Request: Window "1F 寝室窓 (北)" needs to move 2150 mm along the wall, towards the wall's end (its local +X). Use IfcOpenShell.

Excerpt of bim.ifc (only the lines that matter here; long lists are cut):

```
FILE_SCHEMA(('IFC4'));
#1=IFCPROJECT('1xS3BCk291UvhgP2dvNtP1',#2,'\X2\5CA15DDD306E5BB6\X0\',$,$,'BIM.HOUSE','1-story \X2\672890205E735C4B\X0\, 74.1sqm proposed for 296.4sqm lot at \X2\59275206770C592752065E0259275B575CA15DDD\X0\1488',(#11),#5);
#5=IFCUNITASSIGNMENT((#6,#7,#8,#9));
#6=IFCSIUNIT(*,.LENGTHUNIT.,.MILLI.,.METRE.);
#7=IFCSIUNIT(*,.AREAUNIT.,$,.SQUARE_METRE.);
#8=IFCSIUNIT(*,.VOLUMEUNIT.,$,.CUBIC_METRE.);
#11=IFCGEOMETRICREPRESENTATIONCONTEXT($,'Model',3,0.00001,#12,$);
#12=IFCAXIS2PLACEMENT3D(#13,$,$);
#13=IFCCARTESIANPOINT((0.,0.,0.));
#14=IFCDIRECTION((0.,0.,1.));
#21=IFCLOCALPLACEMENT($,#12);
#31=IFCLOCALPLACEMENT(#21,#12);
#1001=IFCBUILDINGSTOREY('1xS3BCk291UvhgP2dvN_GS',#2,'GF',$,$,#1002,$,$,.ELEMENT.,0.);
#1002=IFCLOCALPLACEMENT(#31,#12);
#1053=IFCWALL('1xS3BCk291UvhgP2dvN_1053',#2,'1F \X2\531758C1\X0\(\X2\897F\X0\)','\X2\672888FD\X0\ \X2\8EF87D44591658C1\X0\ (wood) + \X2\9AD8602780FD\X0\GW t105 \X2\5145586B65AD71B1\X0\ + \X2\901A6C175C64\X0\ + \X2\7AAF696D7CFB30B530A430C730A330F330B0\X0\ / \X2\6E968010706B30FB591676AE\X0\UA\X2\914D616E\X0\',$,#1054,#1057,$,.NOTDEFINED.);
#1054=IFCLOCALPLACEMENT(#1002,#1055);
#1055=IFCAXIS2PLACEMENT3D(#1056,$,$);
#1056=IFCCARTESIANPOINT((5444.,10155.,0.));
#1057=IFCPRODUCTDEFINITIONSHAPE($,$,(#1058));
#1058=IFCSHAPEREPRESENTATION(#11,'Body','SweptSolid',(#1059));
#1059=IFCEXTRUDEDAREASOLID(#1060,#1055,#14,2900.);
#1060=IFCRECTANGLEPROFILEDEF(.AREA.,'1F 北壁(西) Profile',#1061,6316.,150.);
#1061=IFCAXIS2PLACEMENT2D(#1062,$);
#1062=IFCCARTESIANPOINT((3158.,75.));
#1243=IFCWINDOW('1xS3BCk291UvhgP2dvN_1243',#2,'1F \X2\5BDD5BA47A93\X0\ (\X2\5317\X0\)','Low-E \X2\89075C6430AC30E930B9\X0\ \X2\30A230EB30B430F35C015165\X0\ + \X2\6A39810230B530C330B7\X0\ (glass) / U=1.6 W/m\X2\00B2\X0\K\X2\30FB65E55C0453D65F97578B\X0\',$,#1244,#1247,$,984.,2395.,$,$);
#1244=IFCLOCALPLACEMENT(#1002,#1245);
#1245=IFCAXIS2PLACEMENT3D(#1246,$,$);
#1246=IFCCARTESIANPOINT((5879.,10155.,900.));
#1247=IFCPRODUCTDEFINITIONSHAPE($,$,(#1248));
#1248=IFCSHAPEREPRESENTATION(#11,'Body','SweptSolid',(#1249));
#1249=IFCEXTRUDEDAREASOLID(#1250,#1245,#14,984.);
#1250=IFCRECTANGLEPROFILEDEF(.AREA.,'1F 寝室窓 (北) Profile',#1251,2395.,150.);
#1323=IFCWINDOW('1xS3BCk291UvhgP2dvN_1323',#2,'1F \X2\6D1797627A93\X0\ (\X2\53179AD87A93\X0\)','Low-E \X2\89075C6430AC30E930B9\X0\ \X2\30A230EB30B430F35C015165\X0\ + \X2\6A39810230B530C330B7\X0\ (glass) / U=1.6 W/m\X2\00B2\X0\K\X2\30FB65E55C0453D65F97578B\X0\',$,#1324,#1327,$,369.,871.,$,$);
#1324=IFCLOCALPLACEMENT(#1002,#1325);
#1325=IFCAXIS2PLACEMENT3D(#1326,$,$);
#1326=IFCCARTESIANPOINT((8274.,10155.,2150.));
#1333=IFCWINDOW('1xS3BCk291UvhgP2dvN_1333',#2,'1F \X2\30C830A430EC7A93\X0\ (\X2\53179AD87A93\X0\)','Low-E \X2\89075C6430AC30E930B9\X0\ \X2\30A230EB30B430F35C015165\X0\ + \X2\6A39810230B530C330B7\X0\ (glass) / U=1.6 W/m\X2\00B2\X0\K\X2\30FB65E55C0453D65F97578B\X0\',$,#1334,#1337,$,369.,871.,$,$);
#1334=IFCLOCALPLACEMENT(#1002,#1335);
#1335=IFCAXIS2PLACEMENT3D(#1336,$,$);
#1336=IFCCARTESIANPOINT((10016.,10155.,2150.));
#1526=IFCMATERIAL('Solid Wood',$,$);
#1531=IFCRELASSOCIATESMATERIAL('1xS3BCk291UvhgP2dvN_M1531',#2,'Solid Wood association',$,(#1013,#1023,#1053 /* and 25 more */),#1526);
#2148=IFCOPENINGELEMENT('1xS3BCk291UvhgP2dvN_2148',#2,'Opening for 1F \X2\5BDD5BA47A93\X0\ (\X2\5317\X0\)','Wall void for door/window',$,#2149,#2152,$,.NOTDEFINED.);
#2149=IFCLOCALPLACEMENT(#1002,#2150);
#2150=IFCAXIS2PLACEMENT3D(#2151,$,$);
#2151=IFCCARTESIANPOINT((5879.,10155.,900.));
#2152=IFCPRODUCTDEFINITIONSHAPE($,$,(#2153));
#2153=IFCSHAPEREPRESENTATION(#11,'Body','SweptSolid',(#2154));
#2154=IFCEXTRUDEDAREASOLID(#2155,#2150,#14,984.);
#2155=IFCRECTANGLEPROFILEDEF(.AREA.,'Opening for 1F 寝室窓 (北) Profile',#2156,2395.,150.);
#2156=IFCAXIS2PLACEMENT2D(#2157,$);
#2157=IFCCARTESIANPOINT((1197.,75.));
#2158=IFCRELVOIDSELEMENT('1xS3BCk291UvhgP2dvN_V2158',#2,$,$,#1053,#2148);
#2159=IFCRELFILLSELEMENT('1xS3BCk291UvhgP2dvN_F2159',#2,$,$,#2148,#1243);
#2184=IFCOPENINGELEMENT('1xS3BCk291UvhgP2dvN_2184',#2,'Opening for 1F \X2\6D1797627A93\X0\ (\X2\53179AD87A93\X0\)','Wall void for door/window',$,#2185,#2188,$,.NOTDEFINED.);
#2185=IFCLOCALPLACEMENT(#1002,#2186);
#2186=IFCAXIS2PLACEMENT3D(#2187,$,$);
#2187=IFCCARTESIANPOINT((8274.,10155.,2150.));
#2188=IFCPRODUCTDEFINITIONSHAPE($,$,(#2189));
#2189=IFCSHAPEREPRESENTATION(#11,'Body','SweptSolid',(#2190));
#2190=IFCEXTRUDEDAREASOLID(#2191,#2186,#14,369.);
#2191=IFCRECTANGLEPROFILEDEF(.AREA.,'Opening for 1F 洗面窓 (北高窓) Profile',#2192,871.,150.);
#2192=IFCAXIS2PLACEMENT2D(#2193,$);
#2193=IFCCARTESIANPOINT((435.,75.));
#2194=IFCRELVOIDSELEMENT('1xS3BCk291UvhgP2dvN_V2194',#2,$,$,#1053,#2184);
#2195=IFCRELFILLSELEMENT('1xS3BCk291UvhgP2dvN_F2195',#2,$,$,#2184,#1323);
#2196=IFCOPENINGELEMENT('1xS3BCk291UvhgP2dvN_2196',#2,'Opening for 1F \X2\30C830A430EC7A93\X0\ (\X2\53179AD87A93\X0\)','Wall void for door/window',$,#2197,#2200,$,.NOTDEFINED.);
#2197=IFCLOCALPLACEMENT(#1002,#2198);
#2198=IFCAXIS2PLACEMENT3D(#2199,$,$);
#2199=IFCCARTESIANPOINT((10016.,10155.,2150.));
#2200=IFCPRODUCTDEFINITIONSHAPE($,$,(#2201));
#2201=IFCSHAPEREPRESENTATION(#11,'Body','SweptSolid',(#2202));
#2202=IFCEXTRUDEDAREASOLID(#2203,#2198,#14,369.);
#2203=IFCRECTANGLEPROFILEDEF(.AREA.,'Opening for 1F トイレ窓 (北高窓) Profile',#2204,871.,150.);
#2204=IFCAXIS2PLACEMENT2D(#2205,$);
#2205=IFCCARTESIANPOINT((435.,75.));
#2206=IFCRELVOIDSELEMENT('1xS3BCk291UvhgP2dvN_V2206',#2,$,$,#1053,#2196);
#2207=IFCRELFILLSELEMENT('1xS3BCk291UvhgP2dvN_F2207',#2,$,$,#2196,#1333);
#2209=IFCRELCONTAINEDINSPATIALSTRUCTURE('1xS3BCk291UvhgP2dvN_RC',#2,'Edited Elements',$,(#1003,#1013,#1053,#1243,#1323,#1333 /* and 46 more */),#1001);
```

```python
import ifcopenshell
import ifcopenshell.api.geometry
import ifcopenshell.util.placement

model = ifcopenshell.open("bim.ifc")

window = model.by_guid("1xS3BCk291UvhgP2dvN_1243")
opening = window.FillsVoids[0].RelatingOpeningElement
wall = opening.VoidsElements[0].RelatingBuildingElement

wall_matrix = ifcopenshell.util.placement.get_local_placement(wall.ObjectPlacement)
shift = wall_matrix[:3, 0] * 2150.0
before = ifcopenshell.util.placement.get_local_placement(window.ObjectPlacement)[:3, 3].copy()

# The window is not placed relative to its opening, so move both.
for product in (opening, window):
    matrix = ifcopenshell.util.placement.get_local_placement(product.ObjectPlacement)
    matrix[:3, 3] += shift
    ifcopenshell.api.geometry.edit_object_placement(model, product=product, matrix=matrix, is_si=False)

after = ifcopenshell.util.placement.get_local_placement(window.ObjectPlacement)[:3, 3]
print("window moved by", (after - before).round(3) + 0.0)

model.write("bim_v2.ifc")
```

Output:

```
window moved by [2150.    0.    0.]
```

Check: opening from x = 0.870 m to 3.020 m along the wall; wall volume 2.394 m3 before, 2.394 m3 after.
